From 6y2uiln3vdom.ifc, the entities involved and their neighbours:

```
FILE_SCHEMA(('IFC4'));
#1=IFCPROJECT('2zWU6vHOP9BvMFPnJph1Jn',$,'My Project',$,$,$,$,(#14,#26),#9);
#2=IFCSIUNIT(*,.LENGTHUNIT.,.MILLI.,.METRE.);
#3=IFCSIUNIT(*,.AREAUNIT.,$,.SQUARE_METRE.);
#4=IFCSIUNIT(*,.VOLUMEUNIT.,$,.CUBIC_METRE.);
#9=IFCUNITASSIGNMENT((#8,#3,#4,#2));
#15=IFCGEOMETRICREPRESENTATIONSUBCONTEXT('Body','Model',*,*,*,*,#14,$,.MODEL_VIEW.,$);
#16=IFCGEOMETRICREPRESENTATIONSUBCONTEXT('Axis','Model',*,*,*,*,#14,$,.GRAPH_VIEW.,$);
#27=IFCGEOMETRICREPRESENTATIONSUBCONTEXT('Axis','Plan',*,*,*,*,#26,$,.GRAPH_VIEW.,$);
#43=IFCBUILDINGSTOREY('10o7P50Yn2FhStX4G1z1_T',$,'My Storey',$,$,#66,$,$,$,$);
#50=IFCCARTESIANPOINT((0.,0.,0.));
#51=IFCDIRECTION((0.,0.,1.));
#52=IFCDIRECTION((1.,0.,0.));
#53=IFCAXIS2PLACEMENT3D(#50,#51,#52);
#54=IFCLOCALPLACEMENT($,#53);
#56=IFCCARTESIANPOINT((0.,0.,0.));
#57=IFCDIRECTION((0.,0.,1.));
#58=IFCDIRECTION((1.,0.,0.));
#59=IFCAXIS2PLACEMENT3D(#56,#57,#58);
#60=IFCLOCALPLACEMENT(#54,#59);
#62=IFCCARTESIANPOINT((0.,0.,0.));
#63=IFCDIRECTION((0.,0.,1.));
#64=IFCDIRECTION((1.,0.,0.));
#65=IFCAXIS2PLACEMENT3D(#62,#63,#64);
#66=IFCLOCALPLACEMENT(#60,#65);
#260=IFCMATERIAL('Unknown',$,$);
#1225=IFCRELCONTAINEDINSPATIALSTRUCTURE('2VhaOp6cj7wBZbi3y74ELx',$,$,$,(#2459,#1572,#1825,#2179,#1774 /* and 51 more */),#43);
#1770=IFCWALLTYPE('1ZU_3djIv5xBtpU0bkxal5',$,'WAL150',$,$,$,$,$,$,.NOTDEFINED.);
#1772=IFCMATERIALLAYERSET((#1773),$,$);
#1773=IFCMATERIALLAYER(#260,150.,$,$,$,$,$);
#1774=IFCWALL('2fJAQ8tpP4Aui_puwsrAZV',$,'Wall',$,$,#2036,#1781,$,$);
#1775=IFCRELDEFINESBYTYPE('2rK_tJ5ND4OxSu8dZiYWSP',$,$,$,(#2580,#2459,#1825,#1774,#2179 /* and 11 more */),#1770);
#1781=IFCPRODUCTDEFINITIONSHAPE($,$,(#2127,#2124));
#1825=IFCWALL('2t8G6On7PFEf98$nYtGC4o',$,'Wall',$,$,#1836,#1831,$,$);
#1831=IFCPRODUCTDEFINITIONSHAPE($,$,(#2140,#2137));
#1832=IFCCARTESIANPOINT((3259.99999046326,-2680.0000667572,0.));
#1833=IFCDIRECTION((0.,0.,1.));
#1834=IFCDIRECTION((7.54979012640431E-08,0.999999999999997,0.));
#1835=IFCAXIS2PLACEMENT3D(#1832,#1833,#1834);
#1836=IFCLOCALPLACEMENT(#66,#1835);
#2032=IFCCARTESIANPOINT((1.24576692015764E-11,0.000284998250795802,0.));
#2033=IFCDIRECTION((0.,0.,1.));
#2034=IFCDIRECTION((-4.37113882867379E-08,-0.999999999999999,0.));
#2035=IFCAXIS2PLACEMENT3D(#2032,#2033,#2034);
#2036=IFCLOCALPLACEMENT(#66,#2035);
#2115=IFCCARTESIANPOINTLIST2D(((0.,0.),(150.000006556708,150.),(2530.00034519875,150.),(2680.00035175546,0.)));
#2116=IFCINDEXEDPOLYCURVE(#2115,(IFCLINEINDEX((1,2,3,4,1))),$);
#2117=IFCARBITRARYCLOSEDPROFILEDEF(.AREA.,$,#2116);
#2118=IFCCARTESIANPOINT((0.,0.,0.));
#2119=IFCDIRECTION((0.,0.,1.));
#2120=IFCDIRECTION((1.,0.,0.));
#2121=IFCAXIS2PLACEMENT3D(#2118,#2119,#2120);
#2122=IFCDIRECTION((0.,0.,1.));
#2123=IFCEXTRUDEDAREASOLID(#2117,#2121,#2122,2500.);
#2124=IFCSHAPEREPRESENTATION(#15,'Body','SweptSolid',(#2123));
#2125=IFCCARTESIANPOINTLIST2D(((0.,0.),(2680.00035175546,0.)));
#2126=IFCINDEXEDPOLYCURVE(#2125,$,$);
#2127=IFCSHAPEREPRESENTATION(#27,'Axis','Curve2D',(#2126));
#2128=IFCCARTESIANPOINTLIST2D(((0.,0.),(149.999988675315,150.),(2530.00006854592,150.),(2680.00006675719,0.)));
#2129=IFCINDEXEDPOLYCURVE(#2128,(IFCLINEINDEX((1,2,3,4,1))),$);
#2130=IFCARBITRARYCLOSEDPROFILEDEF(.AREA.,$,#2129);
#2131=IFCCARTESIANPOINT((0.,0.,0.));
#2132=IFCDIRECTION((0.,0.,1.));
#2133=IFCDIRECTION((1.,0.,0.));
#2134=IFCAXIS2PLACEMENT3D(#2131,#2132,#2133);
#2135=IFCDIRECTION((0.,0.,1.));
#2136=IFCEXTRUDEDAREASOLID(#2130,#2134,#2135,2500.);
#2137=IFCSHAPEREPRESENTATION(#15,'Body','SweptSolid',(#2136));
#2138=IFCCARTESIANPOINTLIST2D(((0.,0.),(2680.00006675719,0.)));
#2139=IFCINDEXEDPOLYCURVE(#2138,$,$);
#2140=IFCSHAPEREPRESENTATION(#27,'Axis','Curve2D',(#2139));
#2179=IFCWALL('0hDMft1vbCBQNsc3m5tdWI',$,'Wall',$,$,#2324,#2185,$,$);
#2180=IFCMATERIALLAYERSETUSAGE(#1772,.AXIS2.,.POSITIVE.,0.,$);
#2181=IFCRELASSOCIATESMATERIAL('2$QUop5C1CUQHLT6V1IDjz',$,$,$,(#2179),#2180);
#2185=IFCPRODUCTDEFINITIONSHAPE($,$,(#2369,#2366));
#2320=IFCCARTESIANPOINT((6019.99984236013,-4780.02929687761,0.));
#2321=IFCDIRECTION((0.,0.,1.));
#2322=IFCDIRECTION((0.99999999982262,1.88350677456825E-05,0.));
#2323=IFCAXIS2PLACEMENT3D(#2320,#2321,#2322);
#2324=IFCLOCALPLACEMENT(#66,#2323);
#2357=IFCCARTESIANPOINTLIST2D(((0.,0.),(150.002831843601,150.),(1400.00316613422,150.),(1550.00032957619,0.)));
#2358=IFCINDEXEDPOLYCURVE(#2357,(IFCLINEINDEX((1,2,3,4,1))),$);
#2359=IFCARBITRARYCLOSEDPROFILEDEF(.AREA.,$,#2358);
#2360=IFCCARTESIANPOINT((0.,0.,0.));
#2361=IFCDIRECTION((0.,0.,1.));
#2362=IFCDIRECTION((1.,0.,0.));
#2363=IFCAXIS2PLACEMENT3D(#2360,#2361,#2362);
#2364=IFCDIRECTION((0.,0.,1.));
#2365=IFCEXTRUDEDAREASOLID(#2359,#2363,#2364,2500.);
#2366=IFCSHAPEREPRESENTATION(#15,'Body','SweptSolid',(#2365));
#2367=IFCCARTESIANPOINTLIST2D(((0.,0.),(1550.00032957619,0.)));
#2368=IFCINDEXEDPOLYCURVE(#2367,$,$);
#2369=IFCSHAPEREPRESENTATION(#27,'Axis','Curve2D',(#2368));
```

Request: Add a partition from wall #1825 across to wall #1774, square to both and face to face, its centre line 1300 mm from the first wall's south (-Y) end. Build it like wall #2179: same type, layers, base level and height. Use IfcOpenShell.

```python
import numpy as np
import ifcopenshell
import ifcopenshell.api.geometry
import ifcopenshell.api.material
import ifcopenshell.api.pset
import ifcopenshell.api.root
import ifcopenshell.api.spatial
import ifcopenshell.api.type
import ifcopenshell.geom
import ifcopenshell.util.element
import ifcopenshell.util.placement
import ifcopenshell.util.representation
import ifcopenshell.util.shape
import ifcopenshell.util.unit

model = ifcopenshell.open("6y2uiln3vdom.ifc")
unit_scale = ifcopenshell.util.unit.calculate_unit_scale(model)
settings = ifcopenshell.geom.settings()
settings.set("use-world-coords", True)

start_wall = model.by_guid("2t8G6On7PFEf98$nYtGC4o")
end_wall = model.by_id(1774)
like = model.by_guid("0hDMft1vbCBQNsc3m5tdWI")
matrix = ifcopenshell.util.placement.get_local_placement(start_wall.ObjectPlacement)
matrix[:3, 3] *= unit_scale


def extent(element):
    """Bounding box in the first wall's axes, in metres."""
    shape = ifcopenshell.geom.create_shape(settings, element)
    points = (ifcopenshell.util.shape.get_vertices(shape.geometry) - matrix[:3, 3]) @ matrix[:3, :3]
    return points.min(axis=0), points.max(axis=0)


y_start = extent(start_wall)[1][1]
y_end = extent(end_wall)[0][1]
like_min, like_max = extent(like)
length, height = float(abs(y_end - y_start)), float(like_max[2] - like_min[2])
layer_set = ifcopenshell.util.element.get_material(like, should_skip_usage=True)
thickness = sum(layer.LayerThickness for layer in layer_set.MaterialLayers) * unit_scale

wall = ifcopenshell.api.root.create_entity(model, ifc_class="IfcWall", name="New partition")
storey = ifcopenshell.util.element.get_container(like)
ifcopenshell.api.spatial.assign_container(model, products=[wall], relating_structure=storey)
ifcopenshell.api.type.assign_type(
    model, related_objects=[wall], relating_type=ifcopenshell.util.element.get_type(like), should_map_representations=False
)
rel = ifcopenshell.api.material.assign_material(
    model, products=[wall], type="IfcMaterialLayerSetUsage", material=layer_set
)
rel.RelatingMaterial.OffsetFromReferenceLine = -thickness / 2 / unit_scale
pset = ifcopenshell.api.pset.add_pset(model, product=wall, name="Pset_WallCommon")
ifcopenshell.api.pset.edit_pset(model, pset=pset, properties={"IsExternal": False, "LoadBearing": False})

# The axis runs down the middle of the wall.
axis = ifcopenshell.api.geometry.add_axis_representation(
    model, context=ifcopenshell.util.representation.get_context(model, "Model", "Axis"), axis=[(0.0, 0.0), (length, 0.0)]
)
body = ifcopenshell.api.geometry.add_wall_representation(
    model,
    context=ifcopenshell.util.representation.get_context(model, "Model", "Body", "MODEL_VIEW"),
    length=length,
    height=height,
    thickness=thickness,
    offset=-thickness / 2,
)
for representation in (axis, body):
    ifcopenshell.api.geometry.assign_representation(model, product=wall, representation=representation)

placement = matrix @ ifcopenshell.util.placement.rotation(90, "Z")
placement[:, 3] = matrix @ np.array([extent(start_wall)[0][0] + 1.3, y_start, like_min[2], 1.0])
ifcopenshell.api.geometry.edit_object_placement(model, product=wall, matrix=placement)

print(f"partition {length:.3f} m long, {height:.3f} m high, {thickness:.3f} m thick")

model.write("6y2uiln3vdom-out.ifc")
```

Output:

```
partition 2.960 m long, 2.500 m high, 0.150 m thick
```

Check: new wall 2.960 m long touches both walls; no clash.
